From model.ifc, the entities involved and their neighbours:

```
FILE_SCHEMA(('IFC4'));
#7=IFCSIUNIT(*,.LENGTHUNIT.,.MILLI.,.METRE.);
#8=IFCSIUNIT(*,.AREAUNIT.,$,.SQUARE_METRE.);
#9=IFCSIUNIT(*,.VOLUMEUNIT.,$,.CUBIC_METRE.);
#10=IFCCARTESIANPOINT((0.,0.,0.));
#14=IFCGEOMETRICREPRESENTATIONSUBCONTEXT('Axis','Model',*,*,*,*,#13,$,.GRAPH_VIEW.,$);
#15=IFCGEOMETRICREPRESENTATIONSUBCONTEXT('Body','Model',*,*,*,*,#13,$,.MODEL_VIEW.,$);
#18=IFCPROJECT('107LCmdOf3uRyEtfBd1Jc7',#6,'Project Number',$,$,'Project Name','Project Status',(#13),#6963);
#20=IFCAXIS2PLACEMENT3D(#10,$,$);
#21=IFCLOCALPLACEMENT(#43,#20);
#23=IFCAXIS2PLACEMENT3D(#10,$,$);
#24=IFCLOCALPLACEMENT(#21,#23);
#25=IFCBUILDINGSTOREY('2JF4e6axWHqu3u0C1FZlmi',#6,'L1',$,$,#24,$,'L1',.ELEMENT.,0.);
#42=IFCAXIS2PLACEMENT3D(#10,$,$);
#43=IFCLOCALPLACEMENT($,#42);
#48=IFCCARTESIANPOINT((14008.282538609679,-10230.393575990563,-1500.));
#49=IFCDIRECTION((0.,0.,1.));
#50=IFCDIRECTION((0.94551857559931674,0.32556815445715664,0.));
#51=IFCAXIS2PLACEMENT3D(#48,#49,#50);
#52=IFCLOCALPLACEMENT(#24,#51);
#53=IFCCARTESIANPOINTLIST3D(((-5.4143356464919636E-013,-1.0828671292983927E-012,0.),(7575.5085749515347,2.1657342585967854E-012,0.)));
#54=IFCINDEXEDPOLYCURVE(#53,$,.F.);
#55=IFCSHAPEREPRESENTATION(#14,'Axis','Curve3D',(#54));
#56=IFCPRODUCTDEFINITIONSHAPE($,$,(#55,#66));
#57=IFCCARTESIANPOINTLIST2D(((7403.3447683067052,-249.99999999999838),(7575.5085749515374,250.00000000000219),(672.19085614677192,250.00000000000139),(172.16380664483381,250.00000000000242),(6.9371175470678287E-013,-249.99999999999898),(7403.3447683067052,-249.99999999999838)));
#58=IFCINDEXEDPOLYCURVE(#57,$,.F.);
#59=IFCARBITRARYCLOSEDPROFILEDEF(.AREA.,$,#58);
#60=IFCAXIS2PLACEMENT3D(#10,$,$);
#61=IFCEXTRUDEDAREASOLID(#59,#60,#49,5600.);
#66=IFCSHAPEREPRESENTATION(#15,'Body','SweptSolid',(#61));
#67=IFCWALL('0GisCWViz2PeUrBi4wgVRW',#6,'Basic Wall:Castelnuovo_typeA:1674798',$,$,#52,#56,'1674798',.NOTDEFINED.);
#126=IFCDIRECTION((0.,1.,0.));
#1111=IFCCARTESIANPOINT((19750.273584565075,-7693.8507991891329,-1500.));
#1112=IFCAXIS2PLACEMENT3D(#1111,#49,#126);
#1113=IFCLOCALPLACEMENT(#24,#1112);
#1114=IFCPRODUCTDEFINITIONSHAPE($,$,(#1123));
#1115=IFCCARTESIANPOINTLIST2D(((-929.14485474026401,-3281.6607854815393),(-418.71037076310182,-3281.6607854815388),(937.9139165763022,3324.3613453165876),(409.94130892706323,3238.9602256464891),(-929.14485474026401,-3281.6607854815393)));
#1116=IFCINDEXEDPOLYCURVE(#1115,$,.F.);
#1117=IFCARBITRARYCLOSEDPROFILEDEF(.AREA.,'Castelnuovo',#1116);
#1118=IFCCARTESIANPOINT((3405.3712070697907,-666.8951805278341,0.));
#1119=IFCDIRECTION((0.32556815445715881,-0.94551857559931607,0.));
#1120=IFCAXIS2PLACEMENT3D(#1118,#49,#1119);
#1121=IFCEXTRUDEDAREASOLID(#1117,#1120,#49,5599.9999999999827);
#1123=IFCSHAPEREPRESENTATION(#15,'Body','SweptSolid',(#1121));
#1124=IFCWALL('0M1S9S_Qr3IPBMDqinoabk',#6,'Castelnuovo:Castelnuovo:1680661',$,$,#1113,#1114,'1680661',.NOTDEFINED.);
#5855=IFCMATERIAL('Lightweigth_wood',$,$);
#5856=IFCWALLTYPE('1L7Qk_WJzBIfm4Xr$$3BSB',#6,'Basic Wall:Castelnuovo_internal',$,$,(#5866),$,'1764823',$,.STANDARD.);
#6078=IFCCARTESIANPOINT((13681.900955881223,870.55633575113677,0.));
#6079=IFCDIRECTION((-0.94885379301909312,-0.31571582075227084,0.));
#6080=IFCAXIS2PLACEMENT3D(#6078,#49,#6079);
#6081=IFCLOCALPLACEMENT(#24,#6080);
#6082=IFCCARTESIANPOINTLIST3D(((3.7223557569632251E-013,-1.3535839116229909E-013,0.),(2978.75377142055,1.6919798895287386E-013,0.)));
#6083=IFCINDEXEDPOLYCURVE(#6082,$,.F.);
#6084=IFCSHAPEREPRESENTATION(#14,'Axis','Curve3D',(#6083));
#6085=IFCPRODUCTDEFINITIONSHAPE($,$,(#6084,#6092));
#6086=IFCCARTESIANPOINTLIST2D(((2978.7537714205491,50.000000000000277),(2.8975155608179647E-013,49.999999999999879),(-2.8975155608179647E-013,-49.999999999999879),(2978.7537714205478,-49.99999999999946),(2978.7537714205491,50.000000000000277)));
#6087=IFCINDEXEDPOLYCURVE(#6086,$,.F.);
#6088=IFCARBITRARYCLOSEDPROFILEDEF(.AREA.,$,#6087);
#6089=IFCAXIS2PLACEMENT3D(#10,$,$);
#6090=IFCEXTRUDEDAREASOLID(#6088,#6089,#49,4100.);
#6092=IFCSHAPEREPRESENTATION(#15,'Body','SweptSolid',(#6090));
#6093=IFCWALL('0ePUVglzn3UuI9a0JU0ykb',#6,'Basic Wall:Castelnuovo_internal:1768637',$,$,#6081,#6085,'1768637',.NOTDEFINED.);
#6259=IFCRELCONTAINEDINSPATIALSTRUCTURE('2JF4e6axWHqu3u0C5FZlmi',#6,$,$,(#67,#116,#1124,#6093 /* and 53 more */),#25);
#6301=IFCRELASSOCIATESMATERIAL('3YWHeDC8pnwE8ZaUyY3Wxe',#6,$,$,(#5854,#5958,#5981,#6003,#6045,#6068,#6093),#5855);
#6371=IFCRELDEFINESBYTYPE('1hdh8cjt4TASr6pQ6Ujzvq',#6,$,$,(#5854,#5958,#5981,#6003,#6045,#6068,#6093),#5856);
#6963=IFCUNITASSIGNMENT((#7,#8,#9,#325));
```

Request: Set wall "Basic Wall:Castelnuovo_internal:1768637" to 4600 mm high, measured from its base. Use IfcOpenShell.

```python
import ifcopenshell
import ifcopenshell.geom
import ifcopenshell.util.representation
import ifcopenshell.util.shape
import ifcopenshell.util.unit

model = ifcopenshell.open("model.ifc")
unit_scale = ifcopenshell.util.unit.calculate_unit_scale(model)
settings = ifcopenshell.geom.settings()


def volume(element):
    """Net volume in cubic metres, openings subtracted."""
    shape = ifcopenshell.geom.create_shape(settings, element)
    return ifcopenshell.util.shape.get_volume(shape.geometry)


wall = model.by_guid("0ePUVglzn3UuI9a0JU0ykb")
before = volume(wall)

body = ifcopenshell.util.representation.get_representation(wall, "Model", "Body")
solid = body.Items[0]
old_height = solid.Depth
solid.Depth = 4.6 / unit_scale
after = volume(wall)

print(f"height {old_height:g} -> {solid.Depth:g}, volume {before:.3f} -> {after:.3f} m3")

model.write("model-out.ifc")
```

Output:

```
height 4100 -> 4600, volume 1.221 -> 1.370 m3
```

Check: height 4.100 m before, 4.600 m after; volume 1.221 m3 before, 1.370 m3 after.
